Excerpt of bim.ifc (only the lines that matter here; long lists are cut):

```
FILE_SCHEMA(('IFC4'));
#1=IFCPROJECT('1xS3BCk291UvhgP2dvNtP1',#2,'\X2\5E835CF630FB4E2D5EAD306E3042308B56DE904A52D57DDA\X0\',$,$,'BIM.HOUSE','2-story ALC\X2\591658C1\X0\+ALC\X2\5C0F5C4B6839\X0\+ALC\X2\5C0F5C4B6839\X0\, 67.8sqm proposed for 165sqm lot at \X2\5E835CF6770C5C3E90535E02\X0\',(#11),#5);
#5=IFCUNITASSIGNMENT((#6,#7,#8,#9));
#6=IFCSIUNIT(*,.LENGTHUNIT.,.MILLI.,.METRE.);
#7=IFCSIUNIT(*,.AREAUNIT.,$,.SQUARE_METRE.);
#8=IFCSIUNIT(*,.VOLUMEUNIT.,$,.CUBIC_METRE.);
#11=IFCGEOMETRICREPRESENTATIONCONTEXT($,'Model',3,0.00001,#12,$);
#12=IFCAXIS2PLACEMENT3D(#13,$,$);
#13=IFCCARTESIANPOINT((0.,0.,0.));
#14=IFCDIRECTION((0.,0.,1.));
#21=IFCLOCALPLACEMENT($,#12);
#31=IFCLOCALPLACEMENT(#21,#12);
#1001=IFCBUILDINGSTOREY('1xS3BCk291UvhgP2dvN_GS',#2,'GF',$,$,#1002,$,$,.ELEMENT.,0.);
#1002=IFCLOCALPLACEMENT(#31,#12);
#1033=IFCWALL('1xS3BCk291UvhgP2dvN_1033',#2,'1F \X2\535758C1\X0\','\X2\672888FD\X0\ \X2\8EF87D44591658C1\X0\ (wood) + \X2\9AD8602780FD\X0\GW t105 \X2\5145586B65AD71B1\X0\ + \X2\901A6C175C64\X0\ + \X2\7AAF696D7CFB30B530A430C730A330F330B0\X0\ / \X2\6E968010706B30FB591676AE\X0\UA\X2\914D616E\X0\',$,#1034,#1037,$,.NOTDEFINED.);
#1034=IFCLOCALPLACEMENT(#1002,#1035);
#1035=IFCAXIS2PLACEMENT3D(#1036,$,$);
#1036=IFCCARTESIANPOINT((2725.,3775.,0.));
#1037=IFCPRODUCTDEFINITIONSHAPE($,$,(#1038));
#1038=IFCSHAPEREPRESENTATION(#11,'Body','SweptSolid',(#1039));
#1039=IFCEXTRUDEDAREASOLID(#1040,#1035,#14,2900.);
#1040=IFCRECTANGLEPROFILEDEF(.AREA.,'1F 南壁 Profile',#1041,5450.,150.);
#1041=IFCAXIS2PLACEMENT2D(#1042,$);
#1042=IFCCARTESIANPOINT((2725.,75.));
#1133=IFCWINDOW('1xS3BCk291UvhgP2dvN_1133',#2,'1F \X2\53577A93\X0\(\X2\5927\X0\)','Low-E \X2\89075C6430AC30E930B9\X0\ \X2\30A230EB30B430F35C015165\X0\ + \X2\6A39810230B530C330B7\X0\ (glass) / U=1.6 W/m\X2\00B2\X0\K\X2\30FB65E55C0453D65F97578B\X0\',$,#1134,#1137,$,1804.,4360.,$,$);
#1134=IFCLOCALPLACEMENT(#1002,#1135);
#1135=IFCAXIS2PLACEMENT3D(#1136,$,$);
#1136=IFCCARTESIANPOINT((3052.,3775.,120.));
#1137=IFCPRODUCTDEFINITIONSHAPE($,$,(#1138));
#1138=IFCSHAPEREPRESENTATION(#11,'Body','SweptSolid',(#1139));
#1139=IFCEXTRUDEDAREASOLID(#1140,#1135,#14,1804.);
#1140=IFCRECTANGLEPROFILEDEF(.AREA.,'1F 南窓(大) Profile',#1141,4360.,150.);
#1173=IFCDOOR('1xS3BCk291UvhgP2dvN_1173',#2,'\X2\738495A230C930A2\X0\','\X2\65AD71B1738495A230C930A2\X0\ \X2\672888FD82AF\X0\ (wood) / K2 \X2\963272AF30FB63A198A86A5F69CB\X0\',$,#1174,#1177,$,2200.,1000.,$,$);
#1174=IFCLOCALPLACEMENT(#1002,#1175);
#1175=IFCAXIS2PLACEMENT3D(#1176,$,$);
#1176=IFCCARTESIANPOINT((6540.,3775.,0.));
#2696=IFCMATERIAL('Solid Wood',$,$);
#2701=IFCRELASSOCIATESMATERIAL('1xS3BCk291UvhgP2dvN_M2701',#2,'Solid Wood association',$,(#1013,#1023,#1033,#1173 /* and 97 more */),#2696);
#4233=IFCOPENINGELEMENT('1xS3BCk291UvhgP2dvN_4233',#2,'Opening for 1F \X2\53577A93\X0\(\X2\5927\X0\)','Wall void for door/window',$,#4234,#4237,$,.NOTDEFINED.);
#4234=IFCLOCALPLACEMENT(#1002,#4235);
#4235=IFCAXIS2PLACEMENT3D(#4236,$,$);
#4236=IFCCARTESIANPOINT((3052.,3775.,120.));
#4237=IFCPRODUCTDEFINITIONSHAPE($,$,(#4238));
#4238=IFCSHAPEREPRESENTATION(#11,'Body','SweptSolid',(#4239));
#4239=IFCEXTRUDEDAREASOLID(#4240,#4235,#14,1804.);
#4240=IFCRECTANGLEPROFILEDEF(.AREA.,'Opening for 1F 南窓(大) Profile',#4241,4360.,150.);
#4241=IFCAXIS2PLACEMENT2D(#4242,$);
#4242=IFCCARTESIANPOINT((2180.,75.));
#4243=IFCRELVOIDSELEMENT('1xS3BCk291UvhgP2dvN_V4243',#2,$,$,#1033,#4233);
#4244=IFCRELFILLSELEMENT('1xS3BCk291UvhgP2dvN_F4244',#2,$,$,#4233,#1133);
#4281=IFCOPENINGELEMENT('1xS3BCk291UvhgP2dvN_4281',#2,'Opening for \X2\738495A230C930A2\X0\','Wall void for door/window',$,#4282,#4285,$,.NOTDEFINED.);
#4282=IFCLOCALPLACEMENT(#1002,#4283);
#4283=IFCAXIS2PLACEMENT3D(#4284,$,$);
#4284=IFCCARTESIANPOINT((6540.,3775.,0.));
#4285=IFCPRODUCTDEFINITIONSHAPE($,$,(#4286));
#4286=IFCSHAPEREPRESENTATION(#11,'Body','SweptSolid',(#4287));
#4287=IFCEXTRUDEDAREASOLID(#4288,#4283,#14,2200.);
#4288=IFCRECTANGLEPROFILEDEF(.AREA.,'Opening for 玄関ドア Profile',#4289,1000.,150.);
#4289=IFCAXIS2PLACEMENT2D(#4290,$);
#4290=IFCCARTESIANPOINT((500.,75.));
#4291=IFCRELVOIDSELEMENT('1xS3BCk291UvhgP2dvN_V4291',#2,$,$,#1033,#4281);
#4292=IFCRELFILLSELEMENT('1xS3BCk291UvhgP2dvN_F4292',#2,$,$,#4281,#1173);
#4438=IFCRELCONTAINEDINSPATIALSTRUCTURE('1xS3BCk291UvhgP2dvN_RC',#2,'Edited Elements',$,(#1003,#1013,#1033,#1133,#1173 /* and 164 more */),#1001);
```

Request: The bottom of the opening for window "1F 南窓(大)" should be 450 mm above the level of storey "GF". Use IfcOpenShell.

```python
import numpy as np
import ifcopenshell
import ifcopenshell.api.geometry
import ifcopenshell.geom
import ifcopenshell.util.element
import ifcopenshell.util.placement
import ifcopenshell.util.shape
import ifcopenshell.util.unit

model = ifcopenshell.open("bim.ifc")
unit_scale = ifcopenshell.util.unit.calculate_unit_scale(model)

window = model.by_guid("1xS3BCk291UvhgP2dvN_1133")
opening = window.FillsVoids[0].RelatingOpeningElement
storey = ifcopenshell.util.element.get_container(window, ifc_class="IfcBuildingStorey")
level = ifcopenshell.util.placement.get_local_placement(storey.ObjectPlacement)[2, 3]

# The opening's origin need not be at the sill, so measure its lowest point.
shape = ifcopenshell.geom.create_shape(ifcopenshell.geom.settings(), opening)
bottom = ifcopenshell.util.shape.get_shape_bottom_elevation(shape, shape.geometry) / unit_scale
dz = level + 0.45 / unit_scale - bottom

shift = np.array([0.0, 0.0, dz])
# The window is not placed relative to its opening, so move both.
for product in (opening, window):
    matrix = ifcopenshell.util.placement.get_local_placement(product.ObjectPlacement)
    matrix[:3, 3] += shift
    ifcopenshell.api.geometry.edit_object_placement(model, product=product, matrix=matrix, is_si=False)

print(f"moved by {dz * unit_scale:+.3f} m")

model.write("bim_rev.ifc")
```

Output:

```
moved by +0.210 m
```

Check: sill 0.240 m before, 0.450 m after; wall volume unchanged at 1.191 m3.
